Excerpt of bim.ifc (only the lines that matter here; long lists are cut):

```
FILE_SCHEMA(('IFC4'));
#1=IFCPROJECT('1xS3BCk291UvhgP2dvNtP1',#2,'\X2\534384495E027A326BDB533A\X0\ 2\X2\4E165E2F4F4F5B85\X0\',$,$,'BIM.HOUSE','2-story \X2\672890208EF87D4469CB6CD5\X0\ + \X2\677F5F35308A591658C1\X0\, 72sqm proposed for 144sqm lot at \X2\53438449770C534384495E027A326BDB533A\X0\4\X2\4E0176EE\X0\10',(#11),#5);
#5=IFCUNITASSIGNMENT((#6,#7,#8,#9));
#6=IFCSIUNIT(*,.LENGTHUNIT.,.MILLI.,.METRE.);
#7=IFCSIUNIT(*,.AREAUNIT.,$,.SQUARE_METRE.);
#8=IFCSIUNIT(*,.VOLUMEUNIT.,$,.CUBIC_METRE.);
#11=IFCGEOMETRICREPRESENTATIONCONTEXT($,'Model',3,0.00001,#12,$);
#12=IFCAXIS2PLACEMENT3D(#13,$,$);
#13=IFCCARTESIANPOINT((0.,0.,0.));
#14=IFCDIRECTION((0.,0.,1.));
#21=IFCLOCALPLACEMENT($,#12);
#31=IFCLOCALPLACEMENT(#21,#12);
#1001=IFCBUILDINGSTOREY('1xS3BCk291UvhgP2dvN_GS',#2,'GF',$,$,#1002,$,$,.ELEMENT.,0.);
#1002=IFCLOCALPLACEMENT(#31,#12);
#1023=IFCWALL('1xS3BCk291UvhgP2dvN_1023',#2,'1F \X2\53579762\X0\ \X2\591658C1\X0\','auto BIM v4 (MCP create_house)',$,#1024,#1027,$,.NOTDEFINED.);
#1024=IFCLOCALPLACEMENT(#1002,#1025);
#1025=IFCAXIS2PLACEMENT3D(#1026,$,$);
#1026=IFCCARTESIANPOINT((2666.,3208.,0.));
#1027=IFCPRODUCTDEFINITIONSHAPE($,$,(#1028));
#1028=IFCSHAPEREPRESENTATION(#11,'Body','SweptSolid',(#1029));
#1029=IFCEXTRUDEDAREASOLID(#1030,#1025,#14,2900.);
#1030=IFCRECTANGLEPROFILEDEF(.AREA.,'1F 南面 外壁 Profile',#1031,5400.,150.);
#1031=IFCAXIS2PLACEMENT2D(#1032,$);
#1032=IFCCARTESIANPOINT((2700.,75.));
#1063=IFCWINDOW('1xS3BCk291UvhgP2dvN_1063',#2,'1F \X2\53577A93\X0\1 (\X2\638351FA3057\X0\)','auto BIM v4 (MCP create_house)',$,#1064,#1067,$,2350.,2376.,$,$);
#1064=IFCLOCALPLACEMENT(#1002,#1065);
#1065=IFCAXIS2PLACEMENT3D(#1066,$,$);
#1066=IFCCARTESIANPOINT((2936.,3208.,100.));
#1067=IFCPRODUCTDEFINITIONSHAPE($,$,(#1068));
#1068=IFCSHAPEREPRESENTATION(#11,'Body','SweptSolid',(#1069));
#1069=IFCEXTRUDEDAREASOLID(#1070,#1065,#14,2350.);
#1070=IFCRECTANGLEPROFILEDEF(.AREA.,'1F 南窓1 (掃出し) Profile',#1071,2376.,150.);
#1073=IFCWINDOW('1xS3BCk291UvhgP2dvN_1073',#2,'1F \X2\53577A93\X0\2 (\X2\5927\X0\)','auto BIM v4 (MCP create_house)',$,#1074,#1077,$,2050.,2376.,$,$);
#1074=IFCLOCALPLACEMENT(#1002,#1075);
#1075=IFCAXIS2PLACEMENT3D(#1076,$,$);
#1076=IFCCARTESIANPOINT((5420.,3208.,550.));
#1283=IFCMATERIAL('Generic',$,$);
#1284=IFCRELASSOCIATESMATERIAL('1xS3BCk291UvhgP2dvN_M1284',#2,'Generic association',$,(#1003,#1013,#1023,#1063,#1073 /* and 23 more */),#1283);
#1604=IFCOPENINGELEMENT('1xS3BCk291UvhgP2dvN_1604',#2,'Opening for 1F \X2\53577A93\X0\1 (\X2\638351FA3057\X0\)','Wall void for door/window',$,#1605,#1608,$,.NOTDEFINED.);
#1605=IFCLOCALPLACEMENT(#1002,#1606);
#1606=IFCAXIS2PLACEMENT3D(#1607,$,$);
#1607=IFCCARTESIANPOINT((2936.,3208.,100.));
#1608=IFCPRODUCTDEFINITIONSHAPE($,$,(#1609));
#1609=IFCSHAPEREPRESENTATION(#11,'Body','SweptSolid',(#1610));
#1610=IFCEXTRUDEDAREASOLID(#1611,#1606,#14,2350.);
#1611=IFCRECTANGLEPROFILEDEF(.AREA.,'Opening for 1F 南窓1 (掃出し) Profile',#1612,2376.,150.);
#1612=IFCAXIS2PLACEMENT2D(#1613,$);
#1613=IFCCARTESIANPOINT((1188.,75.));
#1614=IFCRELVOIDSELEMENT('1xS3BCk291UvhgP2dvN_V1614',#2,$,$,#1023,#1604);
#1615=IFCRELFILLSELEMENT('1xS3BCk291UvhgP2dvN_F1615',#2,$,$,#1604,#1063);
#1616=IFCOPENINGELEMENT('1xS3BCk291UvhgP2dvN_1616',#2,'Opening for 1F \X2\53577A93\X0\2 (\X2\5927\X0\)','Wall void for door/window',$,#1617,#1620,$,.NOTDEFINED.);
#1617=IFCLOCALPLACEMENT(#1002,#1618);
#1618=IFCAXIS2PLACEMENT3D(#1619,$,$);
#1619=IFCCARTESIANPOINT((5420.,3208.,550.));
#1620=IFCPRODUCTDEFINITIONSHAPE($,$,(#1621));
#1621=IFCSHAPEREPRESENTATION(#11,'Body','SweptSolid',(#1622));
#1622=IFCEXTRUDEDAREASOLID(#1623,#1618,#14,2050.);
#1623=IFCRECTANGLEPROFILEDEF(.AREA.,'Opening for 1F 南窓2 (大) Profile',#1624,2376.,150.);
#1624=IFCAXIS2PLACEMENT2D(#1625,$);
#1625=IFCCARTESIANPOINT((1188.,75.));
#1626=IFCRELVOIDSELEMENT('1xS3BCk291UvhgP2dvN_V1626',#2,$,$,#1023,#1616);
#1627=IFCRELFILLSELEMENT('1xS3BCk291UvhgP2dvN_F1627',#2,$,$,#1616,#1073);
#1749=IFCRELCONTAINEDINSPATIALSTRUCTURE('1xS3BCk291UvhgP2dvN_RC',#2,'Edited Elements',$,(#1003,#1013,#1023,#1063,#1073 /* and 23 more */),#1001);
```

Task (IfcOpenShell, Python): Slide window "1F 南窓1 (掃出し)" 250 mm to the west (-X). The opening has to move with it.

```python
import ifcopenshell
import ifcopenshell.api.geometry
import ifcopenshell.util.placement
import ifcopenshell.util.unit

model = ifcopenshell.open("bim.ifc")
unit_scale = ifcopenshell.util.unit.calculate_unit_scale(model)

window = model.by_guid("1xS3BCk291UvhgP2dvN_1063")
opening = window.FillsVoids[0].RelatingOpeningElement
wall = opening.VoidsElements[0].RelatingBuildingElement

wall_matrix = ifcopenshell.util.placement.get_local_placement(wall.ObjectPlacement)
shift = wall_matrix[:3, 0] * -0.25 / unit_scale
before = ifcopenshell.util.placement.get_local_placement(window.ObjectPlacement)[:3, 3].copy()

# The window is not placed relative to its opening, so move both.
for product in (opening, window):
    matrix = ifcopenshell.util.placement.get_local_placement(product.ObjectPlacement)
    matrix[:3, 3] += shift
    ifcopenshell.api.geometry.edit_object_placement(model, product=product, matrix=matrix, is_si=False)

after = ifcopenshell.util.placement.get_local_placement(window.ObjectPlacement)[:3, 3]
print("window moved by", (after - before).round(3) + 0.0)

model.write("bim_edited.ifc")
```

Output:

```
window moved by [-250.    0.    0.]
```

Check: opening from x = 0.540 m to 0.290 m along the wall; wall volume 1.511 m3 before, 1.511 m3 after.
